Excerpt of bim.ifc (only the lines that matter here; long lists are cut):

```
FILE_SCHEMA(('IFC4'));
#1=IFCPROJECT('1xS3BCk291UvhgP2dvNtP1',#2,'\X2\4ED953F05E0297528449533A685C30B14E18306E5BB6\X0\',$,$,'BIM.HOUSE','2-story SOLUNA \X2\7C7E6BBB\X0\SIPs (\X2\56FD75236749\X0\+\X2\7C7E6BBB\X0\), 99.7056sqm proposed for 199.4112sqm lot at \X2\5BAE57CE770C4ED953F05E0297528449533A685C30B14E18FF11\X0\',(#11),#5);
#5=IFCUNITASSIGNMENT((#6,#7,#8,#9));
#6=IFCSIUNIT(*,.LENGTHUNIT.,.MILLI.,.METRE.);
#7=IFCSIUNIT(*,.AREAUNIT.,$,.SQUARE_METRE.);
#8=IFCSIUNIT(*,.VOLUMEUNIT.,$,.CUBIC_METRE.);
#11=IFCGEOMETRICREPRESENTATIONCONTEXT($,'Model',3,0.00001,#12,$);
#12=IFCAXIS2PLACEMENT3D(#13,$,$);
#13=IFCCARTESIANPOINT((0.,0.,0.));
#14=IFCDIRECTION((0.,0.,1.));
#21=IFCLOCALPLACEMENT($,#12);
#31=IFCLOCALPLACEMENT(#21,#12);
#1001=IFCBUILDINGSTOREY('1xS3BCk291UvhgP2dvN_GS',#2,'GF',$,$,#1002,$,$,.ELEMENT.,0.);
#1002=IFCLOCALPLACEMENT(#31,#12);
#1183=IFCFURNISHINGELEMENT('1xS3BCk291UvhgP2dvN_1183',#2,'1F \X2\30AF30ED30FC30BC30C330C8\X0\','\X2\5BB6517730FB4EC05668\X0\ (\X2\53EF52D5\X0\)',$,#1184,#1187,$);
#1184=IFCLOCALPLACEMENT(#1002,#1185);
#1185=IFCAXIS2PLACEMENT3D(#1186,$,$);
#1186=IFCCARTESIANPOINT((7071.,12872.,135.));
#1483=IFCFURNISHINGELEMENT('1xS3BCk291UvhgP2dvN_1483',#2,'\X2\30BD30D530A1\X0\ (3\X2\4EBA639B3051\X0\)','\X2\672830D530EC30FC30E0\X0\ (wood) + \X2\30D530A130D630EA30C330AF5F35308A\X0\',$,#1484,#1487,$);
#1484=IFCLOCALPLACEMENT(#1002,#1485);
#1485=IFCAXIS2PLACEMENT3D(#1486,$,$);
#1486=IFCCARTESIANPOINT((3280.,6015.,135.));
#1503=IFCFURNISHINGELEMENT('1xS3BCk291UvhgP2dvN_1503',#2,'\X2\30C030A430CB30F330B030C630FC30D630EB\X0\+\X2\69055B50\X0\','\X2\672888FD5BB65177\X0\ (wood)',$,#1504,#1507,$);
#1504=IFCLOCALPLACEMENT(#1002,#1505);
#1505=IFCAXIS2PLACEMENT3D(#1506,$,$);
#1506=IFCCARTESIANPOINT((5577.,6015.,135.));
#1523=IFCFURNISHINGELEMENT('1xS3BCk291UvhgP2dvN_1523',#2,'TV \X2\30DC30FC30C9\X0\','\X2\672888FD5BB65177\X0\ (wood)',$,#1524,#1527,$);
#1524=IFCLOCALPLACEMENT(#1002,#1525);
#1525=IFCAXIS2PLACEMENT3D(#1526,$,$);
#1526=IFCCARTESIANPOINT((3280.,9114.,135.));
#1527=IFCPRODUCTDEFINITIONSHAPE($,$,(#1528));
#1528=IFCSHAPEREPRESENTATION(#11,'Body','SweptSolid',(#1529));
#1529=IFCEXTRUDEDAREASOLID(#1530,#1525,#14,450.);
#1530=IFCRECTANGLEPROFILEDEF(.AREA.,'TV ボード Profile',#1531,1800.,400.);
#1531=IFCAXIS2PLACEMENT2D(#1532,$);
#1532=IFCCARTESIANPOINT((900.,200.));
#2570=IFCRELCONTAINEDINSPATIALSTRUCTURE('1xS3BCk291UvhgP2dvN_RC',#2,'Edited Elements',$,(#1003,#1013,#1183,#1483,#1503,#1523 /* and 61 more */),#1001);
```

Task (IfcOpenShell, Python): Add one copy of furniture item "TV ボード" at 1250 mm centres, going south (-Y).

```python
import numpy as np
import ifcopenshell
import ifcopenshell.api.geometry
import ifcopenshell.api.root
import ifcopenshell.util.element
import ifcopenshell.util.placement
import ifcopenshell.util.unit

model = ifcopenshell.open("bim.ifc")
unit_scale = ifcopenshell.util.unit.calculate_unit_scale(model)


def reuse_history(source, copy):
    """copy_class also copies each property set's owner history, people and application; keep the originals."""
    for rel in copy.IsDefinedBy:
        if rel.is_a("IfcRelDefinesByProperties") and (history := rel.RelatingPropertyDefinition.OwnerHistory):
            rel.RelatingPropertyDefinition.OwnerHistory = source.OwnerHistory
            ifcopenshell.util.element.remove_deep2(model, history)


source = model.by_guid("1xS3BCk291UvhgP2dvN_1523")
base = ifcopenshell.util.placement.get_local_placement(source.ObjectPlacement)
step = np.array([0.0, -1.0, 0.0]) * 1.25 / unit_scale

for i in range(1, 2):
    copy = ifcopenshell.api.root.copy_class(model, product=source)
    copy.Representation = ifcopenshell.util.element.copy_deep(
        model, source.Representation, exclude=["IfcGeometricRepresentationContext", "IfcRepresentationMap"]
    )
    reuse_history(source, copy)
    matrix = base.copy()
    matrix[:3, 3] += i * step
    print("added at", matrix[:3, 3].round(3) + 0.0)
    ifcopenshell.api.geometry.edit_object_placement(model, product=copy, matrix=matrix, is_si=False)

model.write("bim_updated.ifc")
```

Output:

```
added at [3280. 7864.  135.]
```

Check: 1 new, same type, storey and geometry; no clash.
